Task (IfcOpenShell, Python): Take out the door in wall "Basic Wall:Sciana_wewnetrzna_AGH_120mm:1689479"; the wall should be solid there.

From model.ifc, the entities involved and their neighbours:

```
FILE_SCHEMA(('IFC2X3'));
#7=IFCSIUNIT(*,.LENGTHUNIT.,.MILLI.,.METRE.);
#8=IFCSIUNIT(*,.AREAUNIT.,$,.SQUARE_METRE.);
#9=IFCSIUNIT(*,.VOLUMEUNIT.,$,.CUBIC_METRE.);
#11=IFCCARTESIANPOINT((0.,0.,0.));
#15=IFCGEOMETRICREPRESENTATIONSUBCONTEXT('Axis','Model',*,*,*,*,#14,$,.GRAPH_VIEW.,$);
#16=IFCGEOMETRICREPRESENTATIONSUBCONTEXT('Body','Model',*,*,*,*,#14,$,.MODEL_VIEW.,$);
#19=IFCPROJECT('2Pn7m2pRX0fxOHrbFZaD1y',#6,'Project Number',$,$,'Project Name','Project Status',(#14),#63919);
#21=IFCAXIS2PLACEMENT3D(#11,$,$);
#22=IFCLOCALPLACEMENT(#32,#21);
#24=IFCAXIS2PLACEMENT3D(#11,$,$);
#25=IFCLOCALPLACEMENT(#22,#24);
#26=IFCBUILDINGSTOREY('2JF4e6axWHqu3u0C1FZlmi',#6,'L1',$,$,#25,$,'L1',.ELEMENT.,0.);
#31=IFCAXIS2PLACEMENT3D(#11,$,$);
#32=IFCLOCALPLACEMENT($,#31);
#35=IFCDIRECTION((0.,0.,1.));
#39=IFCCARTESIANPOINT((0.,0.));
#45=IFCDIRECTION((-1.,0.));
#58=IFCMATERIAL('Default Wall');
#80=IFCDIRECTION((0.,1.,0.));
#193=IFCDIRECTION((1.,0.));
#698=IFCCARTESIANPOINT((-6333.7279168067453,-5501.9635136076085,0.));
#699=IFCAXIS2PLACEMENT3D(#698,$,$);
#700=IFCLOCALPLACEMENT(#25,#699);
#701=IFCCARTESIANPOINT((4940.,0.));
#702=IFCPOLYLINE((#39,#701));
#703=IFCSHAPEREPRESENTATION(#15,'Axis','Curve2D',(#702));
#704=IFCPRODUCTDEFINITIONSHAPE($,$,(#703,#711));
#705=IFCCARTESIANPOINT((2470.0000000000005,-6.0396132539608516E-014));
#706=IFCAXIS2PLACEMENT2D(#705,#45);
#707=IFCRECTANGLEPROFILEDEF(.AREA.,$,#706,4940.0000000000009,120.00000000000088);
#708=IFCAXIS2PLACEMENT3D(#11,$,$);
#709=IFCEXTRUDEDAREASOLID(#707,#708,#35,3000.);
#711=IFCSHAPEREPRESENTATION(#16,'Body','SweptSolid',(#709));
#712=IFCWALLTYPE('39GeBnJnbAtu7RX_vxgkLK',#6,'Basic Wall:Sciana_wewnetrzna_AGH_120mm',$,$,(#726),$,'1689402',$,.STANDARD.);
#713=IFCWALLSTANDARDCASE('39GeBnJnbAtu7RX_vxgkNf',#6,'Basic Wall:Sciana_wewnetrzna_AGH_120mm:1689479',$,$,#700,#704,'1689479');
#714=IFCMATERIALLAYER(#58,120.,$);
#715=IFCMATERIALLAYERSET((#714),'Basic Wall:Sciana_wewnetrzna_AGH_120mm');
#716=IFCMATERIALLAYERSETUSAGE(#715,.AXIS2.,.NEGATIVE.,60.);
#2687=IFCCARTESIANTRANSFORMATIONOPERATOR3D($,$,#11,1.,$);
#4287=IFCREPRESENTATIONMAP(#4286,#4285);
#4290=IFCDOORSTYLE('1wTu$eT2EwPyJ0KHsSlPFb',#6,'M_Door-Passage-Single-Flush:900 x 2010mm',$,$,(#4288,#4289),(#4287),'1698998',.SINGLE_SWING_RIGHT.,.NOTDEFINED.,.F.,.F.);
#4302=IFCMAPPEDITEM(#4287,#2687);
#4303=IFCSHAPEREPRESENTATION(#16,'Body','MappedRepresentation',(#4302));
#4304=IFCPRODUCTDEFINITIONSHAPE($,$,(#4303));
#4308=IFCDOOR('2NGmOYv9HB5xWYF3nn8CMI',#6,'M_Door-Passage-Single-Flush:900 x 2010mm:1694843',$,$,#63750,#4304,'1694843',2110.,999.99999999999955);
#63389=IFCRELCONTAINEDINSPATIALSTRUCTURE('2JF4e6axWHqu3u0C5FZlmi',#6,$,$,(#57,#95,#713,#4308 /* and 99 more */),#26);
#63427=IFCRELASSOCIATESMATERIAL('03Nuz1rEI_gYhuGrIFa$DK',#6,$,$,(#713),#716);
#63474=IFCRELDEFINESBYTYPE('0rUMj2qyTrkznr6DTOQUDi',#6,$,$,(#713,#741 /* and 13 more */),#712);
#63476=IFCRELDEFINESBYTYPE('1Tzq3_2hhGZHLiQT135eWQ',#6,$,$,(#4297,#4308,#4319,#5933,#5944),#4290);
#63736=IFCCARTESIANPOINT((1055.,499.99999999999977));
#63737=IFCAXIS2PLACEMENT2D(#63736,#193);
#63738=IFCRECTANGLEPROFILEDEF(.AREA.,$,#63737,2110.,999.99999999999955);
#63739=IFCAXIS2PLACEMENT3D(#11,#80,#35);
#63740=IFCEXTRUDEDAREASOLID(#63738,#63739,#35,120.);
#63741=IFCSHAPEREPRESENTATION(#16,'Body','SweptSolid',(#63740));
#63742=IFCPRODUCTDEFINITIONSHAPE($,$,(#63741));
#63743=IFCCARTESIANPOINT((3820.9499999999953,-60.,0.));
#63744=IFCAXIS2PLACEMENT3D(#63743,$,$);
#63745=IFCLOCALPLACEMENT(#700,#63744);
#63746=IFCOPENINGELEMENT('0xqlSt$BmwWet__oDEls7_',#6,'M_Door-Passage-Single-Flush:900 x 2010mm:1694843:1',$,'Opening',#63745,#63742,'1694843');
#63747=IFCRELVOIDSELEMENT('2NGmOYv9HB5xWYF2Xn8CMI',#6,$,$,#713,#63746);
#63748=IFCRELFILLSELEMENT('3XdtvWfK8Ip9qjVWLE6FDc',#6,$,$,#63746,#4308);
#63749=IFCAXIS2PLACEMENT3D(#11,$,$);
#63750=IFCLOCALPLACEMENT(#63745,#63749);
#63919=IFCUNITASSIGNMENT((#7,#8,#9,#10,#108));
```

```python
import ifcopenshell
import ifcopenshell.api.feature
import ifcopenshell.api.root
import ifcopenshell.geom
import ifcopenshell.util.shape

model = ifcopenshell.open("model.ifc")
settings = ifcopenshell.geom.settings()


def volume(element):
    """Net volume in cubic metres, openings subtracted."""
    shape = ifcopenshell.geom.create_shape(settings, element)
    return ifcopenshell.util.shape.get_volume(shape.geometry)


door = model.by_guid("2NGmOYv9HB5xWYF3nn8CMI")
opening = door.FillsVoids[0].RelatingOpeningElement
wall = opening.VoidsElements[0].RelatingBuildingElement
before = volume(wall)

ifcopenshell.api.root.remove_product(model, product=door)
ifcopenshell.api.feature.remove_feature(model, feature=opening)

after = volume(wall)

print(f"wall volume {before:.3f} -> {after:.3f} m3")

model.write("model_edited.ifc")
```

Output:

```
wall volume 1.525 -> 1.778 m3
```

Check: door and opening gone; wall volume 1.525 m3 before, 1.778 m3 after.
